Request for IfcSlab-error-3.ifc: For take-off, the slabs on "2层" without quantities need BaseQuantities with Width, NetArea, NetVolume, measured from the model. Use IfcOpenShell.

First a look at what the model holds.

```python
import ifcopenshell
import ifcopenshell.util.element
import ifcopenshell.util.unit

model = ifcopenshell.open("IfcSlab-error-3.ifc")
print(model.schema)
for unit_type in ("LENGTHUNIT", "AREAUNIT", "VOLUMEUNIT"):
    print(unit_type, ifcopenshell.util.unit.calculate_unit_scale(model, unit_type))
storey = next(s for s in model.by_type("IfcBuildingStorey") if s.Name == "2层")
slabs = [e for e in ifcopenshell.util.element.get_decomposition(storey) if e.is_a("IfcSlab")]
for e in sorted(slabs, key=lambda e: e.id()):
    print(e.id(), e.is_a(), e.Name, list(ifcopenshell.util.element.get_psets(e, qtos_only=True)), sep=" | ")
```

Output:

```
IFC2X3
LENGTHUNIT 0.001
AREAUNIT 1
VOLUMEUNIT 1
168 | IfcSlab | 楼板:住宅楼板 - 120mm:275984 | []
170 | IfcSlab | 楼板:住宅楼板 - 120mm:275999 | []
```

```python
import ifcopenshell
import ifcopenshell.api.pset
import ifcopenshell.geom
import ifcopenshell.util.element
import ifcopenshell.util.shape
import ifcopenshell.util.unit

model = ifcopenshell.open("IfcSlab-error-3.ifc")
unit_scale = ifcopenshell.util.unit.calculate_unit_scale(model)
area_scale = ifcopenshell.util.unit.calculate_unit_scale(model, "AREAUNIT")
volume_scale = ifcopenshell.util.unit.calculate_unit_scale(model, "VOLUMEUNIT")
settings = ifcopenshell.geom.settings()

storey = next(s for s in model.by_type("IfcBuildingStorey") if s.Name == "2层")
slabs = [e for e in ifcopenshell.util.element.get_decomposition(storey) if e.is_a("IfcSlab")]

for e in sorted(slabs, key=lambda e: e.id()):
    if ifcopenshell.util.element.get_psets(e, qtos_only=True, should_inherit=False):
        continue
    # Geometry comes back in metres, in the element's own axes.
    shape = ifcopenshell.geom.create_shape(settings, e)
    values = {
        "Width": ifcopenshell.util.shape.get_z(shape.geometry) / unit_scale,
        "NetArea": ifcopenshell.util.shape.get_footprint_area(shape.geometry) / area_scale,
        "NetVolume": ifcopenshell.util.shape.get_volume(shape.geometry) / volume_scale,
    }
    qto = ifcopenshell.api.pset.add_qto(model, product=e, name="BaseQuantities")
    ifcopenshell.api.pset.edit_qto(model, qto=qto, properties=values)
    print(e.id(), {k: round(v, 3) for k, v in values.items()})

model.write("IfcSlab-error-3_updated.ifc")
```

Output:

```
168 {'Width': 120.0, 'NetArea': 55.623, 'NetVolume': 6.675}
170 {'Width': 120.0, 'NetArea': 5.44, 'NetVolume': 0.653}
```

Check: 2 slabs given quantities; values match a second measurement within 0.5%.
